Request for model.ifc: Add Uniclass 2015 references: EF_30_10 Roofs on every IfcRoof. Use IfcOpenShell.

First a look at what the model holds.

```python
import ifcopenshell

model = ifcopenshell.open("model.ifc")
print(model.schema)
print("classifications:", [c.Name for c in model.by_type("IfcClassification")])
for ifc_class in ("IfcDoor", "IfcRoof", "IfcStair", "IfcWall", "IfcWindow"):
    print(ifc_class, len(model.by_type(ifc_class)))
```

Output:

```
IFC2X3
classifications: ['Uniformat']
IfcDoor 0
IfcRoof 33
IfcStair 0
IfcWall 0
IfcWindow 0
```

```python
import ifcopenshell
import ifcopenshell.api.classification

model = ifcopenshell.open("model.ifc")

# IFC2X3 requires Source and Edition and has no link from the project to the system.
system = model.create_entity("IfcClassification", Source="NBS", Edition="2015", Name="Uniclass 2015")

codes = {
    "IfcRoof": ("EF_30_10", "Roofs"),
}
for ifc_class, (code, name) in codes.items():
    products = model.by_type(ifc_class)
    ifcopenshell.api.classification.add_reference(
        model, products=products, classification=system, identification=code, name=name
    )
    print(code, len(products))

model.write("model_rev.ifc")
```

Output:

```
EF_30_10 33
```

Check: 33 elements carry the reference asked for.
